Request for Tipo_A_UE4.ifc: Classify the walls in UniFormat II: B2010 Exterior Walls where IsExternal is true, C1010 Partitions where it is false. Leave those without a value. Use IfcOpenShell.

First a look at what the model holds.

```python
import ifcopenshell
import ifcopenshell.util.element

model = ifcopenshell.open("Tipo_A_UE4.ifc")
print(model.schema)
print("classifications:", [c.Name for c in model.by_type("IfcClassification")])
values = [ifcopenshell.util.element.get_pset(e, "Pset_WallCommon", "IsExternal") for e in model.by_type("IfcWall")]
for value in (True, False, None):
    print("IsExternal", value, values.count(value))
```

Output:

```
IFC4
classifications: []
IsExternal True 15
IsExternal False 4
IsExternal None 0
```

```python
import ifcopenshell
import ifcopenshell.api.classification
import ifcopenshell.util.element

model = ifcopenshell.open("Tipo_A_UE4.ifc")

system = ifcopenshell.api.classification.add_classification(model, classification="UniFormat II")

walls = model.by_type("IfcWall")
external = {e: ifcopenshell.util.element.get_pset(e, "Pset_WallCommon", "IsExternal") for e in walls}
for flag, code, name in ((True, "B2010", "Exterior Walls"), (False, "C1010", "Partitions")):
    products = [e for e in walls if external[e] is flag]
    ifcopenshell.api.classification.add_reference(
        model, products=products, classification=system, identification=code, name=name
    )
    print(code, len(products))

model.write("Tipo_A_UE4-out.ifc")
```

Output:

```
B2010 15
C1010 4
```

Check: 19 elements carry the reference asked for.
